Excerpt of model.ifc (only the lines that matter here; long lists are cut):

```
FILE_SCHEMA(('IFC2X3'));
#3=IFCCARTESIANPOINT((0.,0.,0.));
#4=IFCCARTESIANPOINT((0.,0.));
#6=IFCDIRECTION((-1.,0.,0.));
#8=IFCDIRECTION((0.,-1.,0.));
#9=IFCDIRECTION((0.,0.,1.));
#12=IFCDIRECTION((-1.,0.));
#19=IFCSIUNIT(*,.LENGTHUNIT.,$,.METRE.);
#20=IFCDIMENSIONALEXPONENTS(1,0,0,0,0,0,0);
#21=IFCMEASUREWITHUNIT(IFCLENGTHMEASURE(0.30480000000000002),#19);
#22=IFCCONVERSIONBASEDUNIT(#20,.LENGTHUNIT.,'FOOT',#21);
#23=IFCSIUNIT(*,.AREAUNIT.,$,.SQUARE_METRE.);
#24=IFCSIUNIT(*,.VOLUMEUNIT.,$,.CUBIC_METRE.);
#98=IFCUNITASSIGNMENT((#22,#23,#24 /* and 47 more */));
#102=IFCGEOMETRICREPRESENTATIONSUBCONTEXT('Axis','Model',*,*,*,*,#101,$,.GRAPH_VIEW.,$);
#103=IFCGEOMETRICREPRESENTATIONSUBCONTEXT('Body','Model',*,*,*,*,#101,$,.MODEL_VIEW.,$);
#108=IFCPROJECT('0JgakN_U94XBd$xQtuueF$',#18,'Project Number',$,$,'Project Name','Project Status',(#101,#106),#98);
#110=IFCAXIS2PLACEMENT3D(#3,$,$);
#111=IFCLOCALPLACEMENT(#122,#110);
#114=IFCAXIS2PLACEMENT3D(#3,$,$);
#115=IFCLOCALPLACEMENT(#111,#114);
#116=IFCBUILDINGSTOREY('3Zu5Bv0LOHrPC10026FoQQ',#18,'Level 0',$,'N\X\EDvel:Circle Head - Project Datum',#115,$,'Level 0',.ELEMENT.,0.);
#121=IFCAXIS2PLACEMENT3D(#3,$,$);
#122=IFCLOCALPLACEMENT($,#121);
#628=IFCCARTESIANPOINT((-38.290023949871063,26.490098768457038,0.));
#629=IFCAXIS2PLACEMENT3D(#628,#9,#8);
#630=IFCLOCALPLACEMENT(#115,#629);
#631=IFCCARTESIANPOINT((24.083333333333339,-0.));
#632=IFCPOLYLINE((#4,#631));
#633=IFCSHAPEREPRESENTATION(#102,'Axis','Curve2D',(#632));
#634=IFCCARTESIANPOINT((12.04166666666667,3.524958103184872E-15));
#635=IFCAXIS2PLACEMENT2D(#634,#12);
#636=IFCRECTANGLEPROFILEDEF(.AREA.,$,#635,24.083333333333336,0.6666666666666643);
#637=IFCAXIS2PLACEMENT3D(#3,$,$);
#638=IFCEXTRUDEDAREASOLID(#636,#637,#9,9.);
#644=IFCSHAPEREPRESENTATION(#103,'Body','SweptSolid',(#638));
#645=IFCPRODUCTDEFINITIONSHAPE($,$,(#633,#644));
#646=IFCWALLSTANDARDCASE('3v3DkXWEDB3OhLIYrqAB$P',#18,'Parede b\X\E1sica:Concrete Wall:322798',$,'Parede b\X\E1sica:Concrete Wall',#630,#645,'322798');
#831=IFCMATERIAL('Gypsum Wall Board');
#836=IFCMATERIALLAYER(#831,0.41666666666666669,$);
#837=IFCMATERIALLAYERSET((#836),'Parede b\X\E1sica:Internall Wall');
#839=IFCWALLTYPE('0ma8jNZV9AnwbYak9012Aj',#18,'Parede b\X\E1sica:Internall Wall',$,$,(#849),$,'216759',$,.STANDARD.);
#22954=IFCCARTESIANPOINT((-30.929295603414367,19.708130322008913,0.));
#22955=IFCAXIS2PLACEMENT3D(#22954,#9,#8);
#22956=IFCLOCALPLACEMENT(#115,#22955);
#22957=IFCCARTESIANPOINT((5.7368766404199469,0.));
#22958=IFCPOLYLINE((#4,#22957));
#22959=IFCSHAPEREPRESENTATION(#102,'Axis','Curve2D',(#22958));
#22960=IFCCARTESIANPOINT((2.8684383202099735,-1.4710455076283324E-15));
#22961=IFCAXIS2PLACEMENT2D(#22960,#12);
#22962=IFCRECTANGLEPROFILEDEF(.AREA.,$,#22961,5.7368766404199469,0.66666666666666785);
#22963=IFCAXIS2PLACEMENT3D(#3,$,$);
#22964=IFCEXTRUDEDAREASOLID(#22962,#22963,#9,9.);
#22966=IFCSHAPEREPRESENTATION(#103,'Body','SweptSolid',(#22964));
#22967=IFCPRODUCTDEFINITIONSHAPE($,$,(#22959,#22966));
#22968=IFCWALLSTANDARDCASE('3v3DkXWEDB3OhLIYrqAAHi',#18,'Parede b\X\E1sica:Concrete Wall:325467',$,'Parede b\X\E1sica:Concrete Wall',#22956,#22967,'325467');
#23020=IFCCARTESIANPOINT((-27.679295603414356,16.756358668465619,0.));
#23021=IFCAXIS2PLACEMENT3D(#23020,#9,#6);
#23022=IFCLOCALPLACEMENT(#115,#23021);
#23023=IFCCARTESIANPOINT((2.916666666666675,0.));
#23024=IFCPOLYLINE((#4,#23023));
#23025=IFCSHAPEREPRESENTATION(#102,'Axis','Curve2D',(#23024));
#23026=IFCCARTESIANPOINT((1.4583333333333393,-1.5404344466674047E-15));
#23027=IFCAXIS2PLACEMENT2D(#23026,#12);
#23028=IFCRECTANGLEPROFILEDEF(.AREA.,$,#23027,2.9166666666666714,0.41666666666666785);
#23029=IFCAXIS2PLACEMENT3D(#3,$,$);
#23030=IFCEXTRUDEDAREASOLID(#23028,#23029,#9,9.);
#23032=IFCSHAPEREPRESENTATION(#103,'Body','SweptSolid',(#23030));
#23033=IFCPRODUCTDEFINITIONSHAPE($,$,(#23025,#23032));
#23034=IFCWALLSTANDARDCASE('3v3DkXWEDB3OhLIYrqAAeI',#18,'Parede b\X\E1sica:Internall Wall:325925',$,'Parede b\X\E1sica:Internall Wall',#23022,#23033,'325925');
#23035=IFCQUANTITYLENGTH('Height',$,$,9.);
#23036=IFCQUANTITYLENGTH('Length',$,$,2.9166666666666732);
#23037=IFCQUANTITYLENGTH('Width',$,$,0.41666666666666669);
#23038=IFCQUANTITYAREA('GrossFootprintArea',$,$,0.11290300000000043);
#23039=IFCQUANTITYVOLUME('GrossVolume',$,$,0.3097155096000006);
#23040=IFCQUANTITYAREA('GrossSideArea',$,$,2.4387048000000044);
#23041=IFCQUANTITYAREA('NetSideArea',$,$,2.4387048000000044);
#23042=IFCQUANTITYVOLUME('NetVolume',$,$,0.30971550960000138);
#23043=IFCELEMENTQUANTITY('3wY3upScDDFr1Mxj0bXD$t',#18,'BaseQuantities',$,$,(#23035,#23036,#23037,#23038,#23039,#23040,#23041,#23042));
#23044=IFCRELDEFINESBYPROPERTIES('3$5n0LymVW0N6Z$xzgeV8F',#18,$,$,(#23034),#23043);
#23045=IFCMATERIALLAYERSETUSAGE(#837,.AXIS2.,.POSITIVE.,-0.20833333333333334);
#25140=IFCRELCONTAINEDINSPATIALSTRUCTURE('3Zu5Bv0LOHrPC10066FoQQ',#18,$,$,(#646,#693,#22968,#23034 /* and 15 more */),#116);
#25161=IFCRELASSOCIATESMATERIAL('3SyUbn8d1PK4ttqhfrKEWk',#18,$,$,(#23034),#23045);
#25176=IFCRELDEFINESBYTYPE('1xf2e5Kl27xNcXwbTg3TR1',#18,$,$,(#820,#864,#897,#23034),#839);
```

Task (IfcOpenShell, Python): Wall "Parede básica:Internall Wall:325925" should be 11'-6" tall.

```python
import ifcopenshell
import ifcopenshell.api.pset
import ifcopenshell.geom
import ifcopenshell.util.element
import ifcopenshell.util.representation
import ifcopenshell.util.shape
import ifcopenshell.util.unit

model = ifcopenshell.open("model.ifc")
unit_scale = ifcopenshell.util.unit.calculate_unit_scale(model)
area_scale = ifcopenshell.util.unit.calculate_unit_scale(model, "AREAUNIT")
volume_scale = ifcopenshell.util.unit.calculate_unit_scale(model, "VOLUMEUNIT")
settings = ifcopenshell.geom.settings()


def volume(element):
    """Net volume in cubic metres, openings subtracted."""
    shape = ifcopenshell.geom.create_shape(settings, element)
    return ifcopenshell.util.shape.get_volume(shape.geometry)


wall = model.by_id(23034)
before = volume(wall)

body = ifcopenshell.util.representation.get_representation(wall, "Model", "Body")
solid = body.Items[0]
old_height = solid.Depth
solid.Depth = 138 * 0.0254 / unit_scale
after = volume(wall)
thickness = 0.127  # wall thickness in metres

# Update the stored height, areas and volumes.
qto = model.by_id(ifcopenshell.util.element.get_pset(wall, "BaseQuantities", should_inherit=False)["id"])
ifcopenshell.api.pset.edit_qto(model, qto=qto, properties={
    "Height": solid.Depth,
    "GrossVolume": ifcopenshell.util.element.get_pset(wall, "BaseQuantities", "GrossVolume") * solid.Depth / old_height,
    "GrossSideArea": ifcopenshell.util.element.get_pset(wall, "BaseQuantities", "GrossSideArea") * solid.Depth / old_height,
    "NetSideArea": after / thickness / area_scale,
    "NetVolume": after / volume_scale,
})

print(f"height {old_height:g} -> {solid.Depth:g}, volume {before:.3f} -> {after:.3f} m3")

model.write("model_rev.ifc")
```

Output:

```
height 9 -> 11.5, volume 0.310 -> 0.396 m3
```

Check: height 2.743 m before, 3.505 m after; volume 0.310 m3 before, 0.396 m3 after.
